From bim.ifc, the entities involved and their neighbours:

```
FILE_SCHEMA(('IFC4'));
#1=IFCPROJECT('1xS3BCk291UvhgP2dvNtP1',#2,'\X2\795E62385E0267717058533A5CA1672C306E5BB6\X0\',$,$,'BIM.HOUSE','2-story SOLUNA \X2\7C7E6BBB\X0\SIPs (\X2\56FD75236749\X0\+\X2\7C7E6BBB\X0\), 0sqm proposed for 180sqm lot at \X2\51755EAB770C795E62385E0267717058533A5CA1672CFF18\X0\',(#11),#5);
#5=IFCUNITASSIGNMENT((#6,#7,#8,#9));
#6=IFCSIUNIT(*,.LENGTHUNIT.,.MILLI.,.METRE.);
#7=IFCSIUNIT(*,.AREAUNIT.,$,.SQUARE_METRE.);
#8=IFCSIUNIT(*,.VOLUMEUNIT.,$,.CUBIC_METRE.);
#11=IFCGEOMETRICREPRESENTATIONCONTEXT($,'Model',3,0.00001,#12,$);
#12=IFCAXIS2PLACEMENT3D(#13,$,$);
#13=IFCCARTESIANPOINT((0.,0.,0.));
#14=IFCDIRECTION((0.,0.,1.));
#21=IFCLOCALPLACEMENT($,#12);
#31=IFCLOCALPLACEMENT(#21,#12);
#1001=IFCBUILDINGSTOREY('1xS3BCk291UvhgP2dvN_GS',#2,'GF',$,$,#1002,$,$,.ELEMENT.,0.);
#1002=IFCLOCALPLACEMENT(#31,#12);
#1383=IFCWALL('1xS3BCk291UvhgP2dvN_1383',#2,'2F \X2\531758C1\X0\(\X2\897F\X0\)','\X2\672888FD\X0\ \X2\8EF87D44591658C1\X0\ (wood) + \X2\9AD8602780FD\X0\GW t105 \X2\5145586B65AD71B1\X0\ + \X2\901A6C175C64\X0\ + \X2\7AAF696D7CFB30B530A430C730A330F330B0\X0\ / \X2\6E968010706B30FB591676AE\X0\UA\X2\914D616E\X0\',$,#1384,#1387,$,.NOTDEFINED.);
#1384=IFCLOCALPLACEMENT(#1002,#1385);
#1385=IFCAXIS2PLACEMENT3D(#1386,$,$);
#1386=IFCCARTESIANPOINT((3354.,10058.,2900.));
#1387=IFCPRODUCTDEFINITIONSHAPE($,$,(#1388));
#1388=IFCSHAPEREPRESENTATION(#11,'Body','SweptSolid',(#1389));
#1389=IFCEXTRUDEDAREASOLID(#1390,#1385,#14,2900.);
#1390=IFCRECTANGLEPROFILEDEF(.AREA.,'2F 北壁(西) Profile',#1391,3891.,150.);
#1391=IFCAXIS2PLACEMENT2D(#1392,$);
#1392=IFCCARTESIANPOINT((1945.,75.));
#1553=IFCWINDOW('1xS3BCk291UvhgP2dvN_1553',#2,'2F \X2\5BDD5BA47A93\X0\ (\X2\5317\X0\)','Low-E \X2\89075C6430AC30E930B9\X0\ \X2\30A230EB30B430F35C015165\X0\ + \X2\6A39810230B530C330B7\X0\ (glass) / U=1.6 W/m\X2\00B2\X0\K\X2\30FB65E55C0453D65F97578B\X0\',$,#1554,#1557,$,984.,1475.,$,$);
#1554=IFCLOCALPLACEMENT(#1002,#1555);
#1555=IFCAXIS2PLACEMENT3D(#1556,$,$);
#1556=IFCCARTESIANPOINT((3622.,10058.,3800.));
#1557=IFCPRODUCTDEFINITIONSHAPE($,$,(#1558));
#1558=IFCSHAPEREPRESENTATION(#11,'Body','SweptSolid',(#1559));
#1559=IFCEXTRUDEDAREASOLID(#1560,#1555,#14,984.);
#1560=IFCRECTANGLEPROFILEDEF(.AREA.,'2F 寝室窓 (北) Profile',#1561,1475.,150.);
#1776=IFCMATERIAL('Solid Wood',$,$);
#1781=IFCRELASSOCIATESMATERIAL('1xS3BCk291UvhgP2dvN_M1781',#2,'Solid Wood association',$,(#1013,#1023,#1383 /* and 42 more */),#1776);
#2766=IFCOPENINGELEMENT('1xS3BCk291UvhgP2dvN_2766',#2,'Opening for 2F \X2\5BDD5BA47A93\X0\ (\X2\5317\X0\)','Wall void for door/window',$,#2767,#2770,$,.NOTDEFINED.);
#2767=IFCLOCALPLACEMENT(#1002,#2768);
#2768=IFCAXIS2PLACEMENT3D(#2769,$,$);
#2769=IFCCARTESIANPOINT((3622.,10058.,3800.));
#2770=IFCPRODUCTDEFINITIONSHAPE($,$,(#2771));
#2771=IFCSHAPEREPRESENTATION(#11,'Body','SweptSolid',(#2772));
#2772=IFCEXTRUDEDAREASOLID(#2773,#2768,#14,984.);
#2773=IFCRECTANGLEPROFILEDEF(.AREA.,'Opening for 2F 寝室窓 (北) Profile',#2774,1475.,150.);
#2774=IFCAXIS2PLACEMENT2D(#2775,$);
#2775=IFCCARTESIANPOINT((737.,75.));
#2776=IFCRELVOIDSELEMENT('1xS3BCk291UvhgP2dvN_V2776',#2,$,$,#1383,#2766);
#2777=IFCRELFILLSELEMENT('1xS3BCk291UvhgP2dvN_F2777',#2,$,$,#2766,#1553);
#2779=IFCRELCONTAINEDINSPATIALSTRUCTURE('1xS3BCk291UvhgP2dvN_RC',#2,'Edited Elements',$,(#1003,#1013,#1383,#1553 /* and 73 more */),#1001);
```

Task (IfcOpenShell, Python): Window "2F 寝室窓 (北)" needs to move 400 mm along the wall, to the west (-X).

```python
import ifcopenshell
import ifcopenshell.api.geometry
import ifcopenshell.util.placement

model = ifcopenshell.open("bim.ifc")

window = model.by_guid("1xS3BCk291UvhgP2dvN_1553")
opening = window.FillsVoids[0].RelatingOpeningElement
wall = opening.VoidsElements[0].RelatingBuildingElement

wall_matrix = ifcopenshell.util.placement.get_local_placement(wall.ObjectPlacement)
shift = wall_matrix[:3, 0] * -400.0
before = ifcopenshell.util.placement.get_local_placement(window.ObjectPlacement)[:3, 3].copy()

# The window is not placed relative to its opening, so move both.
for product in (opening, window):
    matrix = ifcopenshell.util.placement.get_local_placement(product.ObjectPlacement)
    matrix[:3, 3] += shift
    ifcopenshell.api.geometry.edit_object_placement(model, product=product, matrix=matrix, is_si=False)

after = ifcopenshell.util.placement.get_local_placement(window.ObjectPlacement)[:3, 3]
print("window moved by", (after - before).round(3) + 0.0)

model.write("bim_rev.ifc")
```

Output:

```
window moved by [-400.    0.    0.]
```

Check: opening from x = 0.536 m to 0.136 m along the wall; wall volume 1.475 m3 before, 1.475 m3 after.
